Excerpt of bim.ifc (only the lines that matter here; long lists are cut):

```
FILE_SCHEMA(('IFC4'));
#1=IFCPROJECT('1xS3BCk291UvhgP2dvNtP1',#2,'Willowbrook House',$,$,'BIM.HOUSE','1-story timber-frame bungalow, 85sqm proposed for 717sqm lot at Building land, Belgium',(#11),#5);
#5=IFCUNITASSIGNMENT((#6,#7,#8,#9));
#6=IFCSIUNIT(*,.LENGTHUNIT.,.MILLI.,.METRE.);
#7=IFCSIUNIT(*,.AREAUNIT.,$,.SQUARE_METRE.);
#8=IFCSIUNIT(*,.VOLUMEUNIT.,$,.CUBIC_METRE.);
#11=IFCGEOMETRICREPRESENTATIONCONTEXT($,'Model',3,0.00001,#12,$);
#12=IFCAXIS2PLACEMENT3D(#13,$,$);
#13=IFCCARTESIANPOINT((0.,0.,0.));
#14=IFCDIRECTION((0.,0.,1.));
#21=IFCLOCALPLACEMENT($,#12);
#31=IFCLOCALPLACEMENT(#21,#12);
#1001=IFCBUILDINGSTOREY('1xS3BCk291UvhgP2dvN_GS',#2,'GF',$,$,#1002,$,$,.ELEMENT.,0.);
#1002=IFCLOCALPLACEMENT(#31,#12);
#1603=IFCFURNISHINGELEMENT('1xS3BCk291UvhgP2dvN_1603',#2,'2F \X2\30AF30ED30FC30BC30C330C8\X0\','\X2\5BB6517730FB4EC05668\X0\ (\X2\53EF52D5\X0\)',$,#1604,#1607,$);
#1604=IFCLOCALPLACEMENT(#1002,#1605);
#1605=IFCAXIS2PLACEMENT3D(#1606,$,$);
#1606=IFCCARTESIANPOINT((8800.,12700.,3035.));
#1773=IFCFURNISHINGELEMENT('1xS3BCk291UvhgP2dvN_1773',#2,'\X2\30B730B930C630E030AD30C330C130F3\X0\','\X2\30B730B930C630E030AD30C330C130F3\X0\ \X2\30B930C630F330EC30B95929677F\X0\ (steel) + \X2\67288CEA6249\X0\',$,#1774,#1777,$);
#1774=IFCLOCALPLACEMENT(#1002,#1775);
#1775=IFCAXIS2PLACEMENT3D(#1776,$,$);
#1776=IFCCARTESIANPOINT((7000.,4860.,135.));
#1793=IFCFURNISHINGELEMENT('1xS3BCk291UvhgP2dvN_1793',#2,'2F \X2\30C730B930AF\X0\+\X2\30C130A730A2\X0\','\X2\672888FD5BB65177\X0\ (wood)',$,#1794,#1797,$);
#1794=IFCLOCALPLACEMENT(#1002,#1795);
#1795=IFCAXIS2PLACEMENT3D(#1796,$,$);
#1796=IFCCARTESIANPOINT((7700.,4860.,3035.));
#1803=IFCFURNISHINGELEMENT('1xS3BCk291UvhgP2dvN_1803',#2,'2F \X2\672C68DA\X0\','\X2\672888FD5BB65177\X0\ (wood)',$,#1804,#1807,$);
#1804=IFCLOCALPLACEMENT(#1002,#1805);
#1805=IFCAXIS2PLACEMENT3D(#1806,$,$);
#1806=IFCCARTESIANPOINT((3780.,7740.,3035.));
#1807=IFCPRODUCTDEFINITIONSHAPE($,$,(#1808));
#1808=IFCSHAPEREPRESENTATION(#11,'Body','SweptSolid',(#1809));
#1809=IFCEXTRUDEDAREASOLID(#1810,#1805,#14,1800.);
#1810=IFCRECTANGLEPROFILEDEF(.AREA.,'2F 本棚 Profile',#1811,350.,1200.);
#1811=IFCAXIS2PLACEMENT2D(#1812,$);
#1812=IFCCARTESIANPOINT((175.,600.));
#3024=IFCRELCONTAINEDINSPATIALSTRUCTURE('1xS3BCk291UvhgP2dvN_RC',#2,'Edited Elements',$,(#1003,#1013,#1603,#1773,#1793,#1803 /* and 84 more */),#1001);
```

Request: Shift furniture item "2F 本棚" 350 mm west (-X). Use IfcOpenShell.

```python
import ifcopenshell
import ifcopenshell.api.geometry
import ifcopenshell.util.placement
import ifcopenshell.util.unit

model = ifcopenshell.open("bim.ifc")
unit_scale = ifcopenshell.util.unit.calculate_unit_scale(model)

item = model.by_guid("1xS3BCk291UvhgP2dvN_1803")
matrix = ifcopenshell.util.placement.get_local_placement(item.ObjectPlacement)
matrix[0, 3] -= 0.35 / unit_scale
ifcopenshell.api.geometry.edit_object_placement(model, product=item, matrix=matrix, is_si=False)

print(ifcopenshell.util.placement.get_local_placement(item.ObjectPlacement).round(3) + 0.0)

model.write("bim_updated.ifc")
```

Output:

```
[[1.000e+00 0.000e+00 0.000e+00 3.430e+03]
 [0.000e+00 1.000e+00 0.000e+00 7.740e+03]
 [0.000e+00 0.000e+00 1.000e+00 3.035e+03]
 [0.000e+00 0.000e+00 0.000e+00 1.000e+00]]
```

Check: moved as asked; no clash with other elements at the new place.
